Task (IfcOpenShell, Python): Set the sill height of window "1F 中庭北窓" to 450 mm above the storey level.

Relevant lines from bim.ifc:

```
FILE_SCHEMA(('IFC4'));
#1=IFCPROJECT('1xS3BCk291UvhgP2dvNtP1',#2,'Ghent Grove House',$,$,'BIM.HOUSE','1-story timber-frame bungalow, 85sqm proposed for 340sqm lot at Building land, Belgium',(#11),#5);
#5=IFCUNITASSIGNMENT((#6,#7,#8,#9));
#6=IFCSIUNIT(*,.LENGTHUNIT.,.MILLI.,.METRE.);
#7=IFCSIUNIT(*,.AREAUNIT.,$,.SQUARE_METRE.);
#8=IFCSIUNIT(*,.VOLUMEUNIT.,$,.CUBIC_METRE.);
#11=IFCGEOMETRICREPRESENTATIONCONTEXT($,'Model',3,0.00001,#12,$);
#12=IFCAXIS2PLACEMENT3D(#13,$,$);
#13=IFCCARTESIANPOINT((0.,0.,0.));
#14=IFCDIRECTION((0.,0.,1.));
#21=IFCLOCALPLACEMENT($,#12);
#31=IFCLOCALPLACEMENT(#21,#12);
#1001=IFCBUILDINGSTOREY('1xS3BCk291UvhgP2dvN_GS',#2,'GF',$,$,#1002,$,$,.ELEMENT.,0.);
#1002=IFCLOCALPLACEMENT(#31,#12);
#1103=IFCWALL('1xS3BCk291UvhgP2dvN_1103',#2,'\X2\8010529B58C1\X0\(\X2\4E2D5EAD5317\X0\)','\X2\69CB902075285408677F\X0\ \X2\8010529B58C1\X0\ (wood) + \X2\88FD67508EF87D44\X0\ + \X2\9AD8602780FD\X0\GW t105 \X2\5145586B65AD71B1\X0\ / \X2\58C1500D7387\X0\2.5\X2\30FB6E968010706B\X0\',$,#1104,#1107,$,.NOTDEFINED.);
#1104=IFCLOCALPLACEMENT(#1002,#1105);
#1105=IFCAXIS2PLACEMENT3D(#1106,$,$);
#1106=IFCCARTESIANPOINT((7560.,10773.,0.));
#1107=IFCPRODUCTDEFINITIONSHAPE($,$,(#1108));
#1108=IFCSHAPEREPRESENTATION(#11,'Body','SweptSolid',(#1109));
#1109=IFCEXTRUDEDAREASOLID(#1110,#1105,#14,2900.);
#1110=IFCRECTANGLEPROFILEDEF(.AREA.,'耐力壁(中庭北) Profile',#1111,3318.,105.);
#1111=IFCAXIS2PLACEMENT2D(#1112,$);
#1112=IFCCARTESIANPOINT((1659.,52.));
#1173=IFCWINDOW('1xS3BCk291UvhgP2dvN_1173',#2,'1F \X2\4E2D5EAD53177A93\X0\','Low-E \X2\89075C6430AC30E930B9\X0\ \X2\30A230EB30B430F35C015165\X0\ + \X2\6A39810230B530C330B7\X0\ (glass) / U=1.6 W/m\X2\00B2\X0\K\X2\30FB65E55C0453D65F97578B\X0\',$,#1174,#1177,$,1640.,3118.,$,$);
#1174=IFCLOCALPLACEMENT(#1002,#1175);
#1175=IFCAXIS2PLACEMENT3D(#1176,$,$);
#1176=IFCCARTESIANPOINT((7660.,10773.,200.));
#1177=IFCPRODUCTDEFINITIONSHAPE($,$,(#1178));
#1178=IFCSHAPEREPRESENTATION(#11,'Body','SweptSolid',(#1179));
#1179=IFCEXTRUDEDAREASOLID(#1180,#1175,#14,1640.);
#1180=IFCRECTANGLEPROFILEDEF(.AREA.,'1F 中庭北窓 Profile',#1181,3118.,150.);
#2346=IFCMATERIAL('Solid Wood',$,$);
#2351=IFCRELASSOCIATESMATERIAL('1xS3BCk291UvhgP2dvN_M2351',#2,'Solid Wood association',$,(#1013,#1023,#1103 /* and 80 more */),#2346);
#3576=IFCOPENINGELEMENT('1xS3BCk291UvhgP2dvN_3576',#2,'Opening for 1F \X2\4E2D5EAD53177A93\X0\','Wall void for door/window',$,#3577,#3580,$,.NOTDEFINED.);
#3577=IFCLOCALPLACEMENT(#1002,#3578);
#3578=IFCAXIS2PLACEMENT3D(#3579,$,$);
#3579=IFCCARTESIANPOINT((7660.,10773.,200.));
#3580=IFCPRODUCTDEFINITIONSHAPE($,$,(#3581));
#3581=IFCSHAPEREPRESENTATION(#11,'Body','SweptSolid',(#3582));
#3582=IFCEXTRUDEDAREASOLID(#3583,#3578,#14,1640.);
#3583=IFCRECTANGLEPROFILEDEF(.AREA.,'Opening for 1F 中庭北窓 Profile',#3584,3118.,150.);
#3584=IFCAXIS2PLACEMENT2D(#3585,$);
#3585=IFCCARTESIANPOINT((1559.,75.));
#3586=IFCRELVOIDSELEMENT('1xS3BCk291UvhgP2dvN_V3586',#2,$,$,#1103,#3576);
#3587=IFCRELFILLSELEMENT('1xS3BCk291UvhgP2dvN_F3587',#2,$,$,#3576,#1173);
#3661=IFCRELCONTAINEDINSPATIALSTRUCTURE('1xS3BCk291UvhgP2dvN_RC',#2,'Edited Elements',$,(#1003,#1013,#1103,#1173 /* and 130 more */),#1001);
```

```python
import numpy as np
import ifcopenshell
import ifcopenshell.api.geometry
import ifcopenshell.geom
import ifcopenshell.util.element
import ifcopenshell.util.placement
import ifcopenshell.util.shape
import ifcopenshell.util.unit

model = ifcopenshell.open("bim.ifc")
unit_scale = ifcopenshell.util.unit.calculate_unit_scale(model)

window = model.by_guid("1xS3BCk291UvhgP2dvN_1173")
opening = window.FillsVoids[0].RelatingOpeningElement
storey = ifcopenshell.util.element.get_container(window, ifc_class="IfcBuildingStorey")
level = ifcopenshell.util.placement.get_local_placement(storey.ObjectPlacement)[2, 3]

# The opening's origin need not be at the sill, so measure its lowest point.
shape = ifcopenshell.geom.create_shape(ifcopenshell.geom.settings(), opening)
bottom = ifcopenshell.util.shape.get_shape_bottom_elevation(shape, shape.geometry) / unit_scale
dz = level + 0.45 / unit_scale - bottom

shift = np.array([0.0, 0.0, dz])
# The window is not placed relative to its opening, so move both.
for product in (opening, window):
    matrix = ifcopenshell.util.placement.get_local_placement(product.ObjectPlacement)
    matrix[:3, 3] += shift
    ifcopenshell.api.geometry.edit_object_placement(model, product=product, matrix=matrix, is_si=False)

print(f"moved by {dz * unit_scale:+.3f} m")

model.write("bim_updated.ifc")
```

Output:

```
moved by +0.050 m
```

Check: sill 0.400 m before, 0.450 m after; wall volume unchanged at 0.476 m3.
